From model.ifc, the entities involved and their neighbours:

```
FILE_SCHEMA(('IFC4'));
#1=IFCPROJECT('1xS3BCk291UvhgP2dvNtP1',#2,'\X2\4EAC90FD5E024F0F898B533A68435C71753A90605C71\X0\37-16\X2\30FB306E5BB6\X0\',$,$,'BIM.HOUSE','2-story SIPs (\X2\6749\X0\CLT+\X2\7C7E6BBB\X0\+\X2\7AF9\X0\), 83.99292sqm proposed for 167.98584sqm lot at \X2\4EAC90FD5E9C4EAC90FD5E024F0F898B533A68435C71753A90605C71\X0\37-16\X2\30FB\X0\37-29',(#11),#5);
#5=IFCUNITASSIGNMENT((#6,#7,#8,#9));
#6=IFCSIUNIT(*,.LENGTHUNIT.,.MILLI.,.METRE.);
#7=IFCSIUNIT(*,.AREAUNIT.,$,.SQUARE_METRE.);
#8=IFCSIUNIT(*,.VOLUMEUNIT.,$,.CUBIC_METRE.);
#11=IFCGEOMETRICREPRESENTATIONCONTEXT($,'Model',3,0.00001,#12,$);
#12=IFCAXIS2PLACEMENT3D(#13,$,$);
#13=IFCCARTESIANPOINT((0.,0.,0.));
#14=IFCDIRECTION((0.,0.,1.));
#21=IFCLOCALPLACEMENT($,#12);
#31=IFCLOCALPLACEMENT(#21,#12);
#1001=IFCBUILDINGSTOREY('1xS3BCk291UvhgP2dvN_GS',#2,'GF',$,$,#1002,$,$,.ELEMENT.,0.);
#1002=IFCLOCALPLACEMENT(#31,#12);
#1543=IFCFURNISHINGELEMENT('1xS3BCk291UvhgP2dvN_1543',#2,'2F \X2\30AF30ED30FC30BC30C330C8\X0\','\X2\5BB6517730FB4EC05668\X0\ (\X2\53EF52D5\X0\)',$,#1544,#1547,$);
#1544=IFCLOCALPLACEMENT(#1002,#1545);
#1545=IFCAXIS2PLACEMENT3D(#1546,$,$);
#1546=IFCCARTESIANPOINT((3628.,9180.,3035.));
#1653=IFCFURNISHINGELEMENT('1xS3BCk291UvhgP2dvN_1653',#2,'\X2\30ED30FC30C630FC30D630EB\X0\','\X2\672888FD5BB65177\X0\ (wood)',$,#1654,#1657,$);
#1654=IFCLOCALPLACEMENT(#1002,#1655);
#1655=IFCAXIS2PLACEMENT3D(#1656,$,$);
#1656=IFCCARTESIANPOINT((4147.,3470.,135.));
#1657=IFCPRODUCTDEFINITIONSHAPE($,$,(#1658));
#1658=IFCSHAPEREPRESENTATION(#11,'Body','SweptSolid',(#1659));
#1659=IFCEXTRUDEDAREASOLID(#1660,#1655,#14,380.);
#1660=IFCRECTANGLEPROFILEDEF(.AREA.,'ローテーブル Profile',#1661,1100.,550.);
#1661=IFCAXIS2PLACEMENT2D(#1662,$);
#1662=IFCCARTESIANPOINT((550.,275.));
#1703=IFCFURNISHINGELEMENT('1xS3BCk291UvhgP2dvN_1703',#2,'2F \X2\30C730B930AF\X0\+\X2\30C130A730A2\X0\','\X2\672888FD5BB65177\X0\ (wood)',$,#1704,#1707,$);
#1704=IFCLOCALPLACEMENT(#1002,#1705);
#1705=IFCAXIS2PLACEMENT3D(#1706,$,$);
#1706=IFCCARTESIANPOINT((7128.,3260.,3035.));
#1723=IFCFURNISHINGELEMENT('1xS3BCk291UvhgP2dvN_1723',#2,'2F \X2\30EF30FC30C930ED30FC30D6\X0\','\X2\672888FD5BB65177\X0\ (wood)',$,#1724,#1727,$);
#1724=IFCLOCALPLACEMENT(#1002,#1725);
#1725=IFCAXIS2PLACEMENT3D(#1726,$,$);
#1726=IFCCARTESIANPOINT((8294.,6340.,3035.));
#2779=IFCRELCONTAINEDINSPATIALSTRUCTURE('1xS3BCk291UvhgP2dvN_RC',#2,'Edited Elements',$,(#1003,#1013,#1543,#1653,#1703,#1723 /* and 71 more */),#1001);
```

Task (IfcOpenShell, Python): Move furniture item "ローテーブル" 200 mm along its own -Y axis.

```python
import ifcopenshell
import ifcopenshell.api.geometry
import ifcopenshell.util.placement

model = ifcopenshell.open("model.ifc")

item = model.by_id(1653)
matrix = ifcopenshell.util.placement.get_local_placement(item.ObjectPlacement)
matrix[:3, 3] -= matrix[:3, 1] * 200.0
ifcopenshell.api.geometry.edit_object_placement(model, product=item, matrix=matrix, is_si=False)

print(ifcopenshell.util.placement.get_local_placement(item.ObjectPlacement).round(3) + 0.0)

model.write("model_edited.ifc")
```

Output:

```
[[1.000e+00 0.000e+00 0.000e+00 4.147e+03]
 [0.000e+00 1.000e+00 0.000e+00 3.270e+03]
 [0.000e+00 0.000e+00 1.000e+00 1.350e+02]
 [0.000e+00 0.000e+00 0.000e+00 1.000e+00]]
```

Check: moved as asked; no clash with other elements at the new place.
